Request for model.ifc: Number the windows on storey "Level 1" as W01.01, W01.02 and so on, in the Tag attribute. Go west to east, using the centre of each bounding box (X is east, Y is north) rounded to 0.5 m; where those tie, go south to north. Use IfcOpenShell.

First a look at what the model holds.

```python
import ifcopenshell
import ifcopenshell.util.element
import ifcopenshell.util.placement

model = ifcopenshell.open("model.ifc")
print(model.schema)
storey = next(s for s in model.by_type("IfcBuildingStorey") if s.Name == "Level 1")
windows = [e for e in ifcopenshell.util.element.get_decomposition(storey) if e.is_a("IfcWindow")]
for e in sorted(windows, key=lambda e: e.id()):
    origin = ifcopenshell.util.placement.get_local_placement(e.ObjectPlacement)[:3, 3]
    print(e.id(), e.Tag, e.Name, origin.round(2) + 0.0, sep=" | ")
```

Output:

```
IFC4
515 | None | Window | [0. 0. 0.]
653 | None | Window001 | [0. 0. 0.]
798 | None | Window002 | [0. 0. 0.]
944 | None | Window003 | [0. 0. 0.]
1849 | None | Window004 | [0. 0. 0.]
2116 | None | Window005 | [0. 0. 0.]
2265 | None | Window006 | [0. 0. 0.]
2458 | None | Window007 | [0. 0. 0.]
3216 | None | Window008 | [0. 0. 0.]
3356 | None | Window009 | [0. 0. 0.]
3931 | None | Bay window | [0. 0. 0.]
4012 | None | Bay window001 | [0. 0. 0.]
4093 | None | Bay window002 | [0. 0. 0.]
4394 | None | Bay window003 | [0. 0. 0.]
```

```python
import ifcopenshell
import ifcopenshell.geom
import ifcopenshell.util.element
import ifcopenshell.util.shape

model = ifcopenshell.open("model.ifc")
settings = ifcopenshell.geom.settings()
settings.set("use-world-coords", True)


def centre(element):
    shape = ifcopenshell.geom.create_shape(settings, element)
    return ifcopenshell.util.shape.get_bbox_centroid(shape.geometry)


storey = next(s for s in model.by_type("IfcBuildingStorey") if s.Name == "Level 1")
windows = [e for e in ifcopenshell.util.element.get_decomposition(storey) if e.is_a("IfcWindow")]

# Insertion points can sit at a corner or the storey origin, so sort by the geometry (in metres).
centres = {e: centre(e) for e in windows}
windows.sort(key=lambda e: (round(centres[e][0] / 0.5), centres[e][1]))

for i, e in enumerate(windows, start=1):
    number = f"W01.{i:02d}"
    e.Tag = number
    print(e.id(), number)

model.write("model_rev.ifc")
```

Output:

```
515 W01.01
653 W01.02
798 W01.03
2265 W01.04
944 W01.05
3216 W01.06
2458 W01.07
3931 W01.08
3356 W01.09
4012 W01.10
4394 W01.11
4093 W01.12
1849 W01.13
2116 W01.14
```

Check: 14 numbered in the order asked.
